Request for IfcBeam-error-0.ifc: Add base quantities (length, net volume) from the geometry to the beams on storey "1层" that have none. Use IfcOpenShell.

First a look at what the model holds.

```python
import ifcopenshell
import ifcopenshell.util.element
import ifcopenshell.util.unit

model = ifcopenshell.open("IfcBeam-error-0.ifc")
print(model.schema)
for unit_type in ("LENGTHUNIT", "AREAUNIT", "VOLUMEUNIT"):
    print(unit_type, ifcopenshell.util.unit.calculate_unit_scale(model, unit_type))
storey = next(s for s in model.by_type("IfcBuildingStorey") if s.Name == "1层")
beams = [e for e in ifcopenshell.util.element.get_decomposition(storey) if e.is_a("IfcBeam")]
for e in sorted(beams, key=lambda e: e.id()):
    print(e.id(), e.is_a(), e.Name, list(ifcopenshell.util.element.get_psets(e, qtos_only=True)), sep=" | ")
```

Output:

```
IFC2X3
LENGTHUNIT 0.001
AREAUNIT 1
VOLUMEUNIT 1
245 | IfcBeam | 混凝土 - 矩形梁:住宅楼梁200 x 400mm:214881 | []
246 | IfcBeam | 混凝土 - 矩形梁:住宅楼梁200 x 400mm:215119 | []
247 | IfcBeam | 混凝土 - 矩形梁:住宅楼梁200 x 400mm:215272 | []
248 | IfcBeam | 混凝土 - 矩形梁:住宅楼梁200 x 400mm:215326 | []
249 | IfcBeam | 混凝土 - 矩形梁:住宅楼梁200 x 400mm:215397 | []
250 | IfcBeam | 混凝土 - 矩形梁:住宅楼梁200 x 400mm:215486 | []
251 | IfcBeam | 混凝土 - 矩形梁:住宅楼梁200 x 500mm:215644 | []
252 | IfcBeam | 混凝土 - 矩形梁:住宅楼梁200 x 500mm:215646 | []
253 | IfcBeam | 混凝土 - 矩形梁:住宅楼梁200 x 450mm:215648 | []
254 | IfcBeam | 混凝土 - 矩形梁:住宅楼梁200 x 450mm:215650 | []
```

```python
import ifcopenshell
import ifcopenshell.api.pset
import ifcopenshell.geom
import ifcopenshell.util.element
import ifcopenshell.util.shape
import ifcopenshell.util.unit

model = ifcopenshell.open("IfcBeam-error-0.ifc")
unit_scale = ifcopenshell.util.unit.calculate_unit_scale(model)
volume_scale = ifcopenshell.util.unit.calculate_unit_scale(model, "VOLUMEUNIT")
settings = ifcopenshell.geom.settings()

storey = next(s for s in model.by_type("IfcBuildingStorey") if s.Name == "1层")
beams = [e for e in ifcopenshell.util.element.get_decomposition(storey) if e.is_a("IfcBeam")]

for e in sorted(beams, key=lambda e: e.id()):
    if ifcopenshell.util.element.get_psets(e, qtos_only=True, should_inherit=False):
        continue
    # Geometry comes back in metres, in the element's own axes.
    shape = ifcopenshell.geom.create_shape(settings, e)
    values = {
        "Length": ifcopenshell.util.shape.get_max_xyz(shape.geometry) / unit_scale,
        "NetVolume": ifcopenshell.util.shape.get_volume(shape.geometry) / volume_scale,
    }
    qto = ifcopenshell.api.pset.add_qto(model, product=e, name="BaseQuantities")
    ifcopenshell.api.pset.edit_qto(model, qto=qto, properties=values)
    print(e.id(), {k: round(v, 3) for k, v in values.items()})

model.write("IfcBeam-error-0_v2.ifc")
```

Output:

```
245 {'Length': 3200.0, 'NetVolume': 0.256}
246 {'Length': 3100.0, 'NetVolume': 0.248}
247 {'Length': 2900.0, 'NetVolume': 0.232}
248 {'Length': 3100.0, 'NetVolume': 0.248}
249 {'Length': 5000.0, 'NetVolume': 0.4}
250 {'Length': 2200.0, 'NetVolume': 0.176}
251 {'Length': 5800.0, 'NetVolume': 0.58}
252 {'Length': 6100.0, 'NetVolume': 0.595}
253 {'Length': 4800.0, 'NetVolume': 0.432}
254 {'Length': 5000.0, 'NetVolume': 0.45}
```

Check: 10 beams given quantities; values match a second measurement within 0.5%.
